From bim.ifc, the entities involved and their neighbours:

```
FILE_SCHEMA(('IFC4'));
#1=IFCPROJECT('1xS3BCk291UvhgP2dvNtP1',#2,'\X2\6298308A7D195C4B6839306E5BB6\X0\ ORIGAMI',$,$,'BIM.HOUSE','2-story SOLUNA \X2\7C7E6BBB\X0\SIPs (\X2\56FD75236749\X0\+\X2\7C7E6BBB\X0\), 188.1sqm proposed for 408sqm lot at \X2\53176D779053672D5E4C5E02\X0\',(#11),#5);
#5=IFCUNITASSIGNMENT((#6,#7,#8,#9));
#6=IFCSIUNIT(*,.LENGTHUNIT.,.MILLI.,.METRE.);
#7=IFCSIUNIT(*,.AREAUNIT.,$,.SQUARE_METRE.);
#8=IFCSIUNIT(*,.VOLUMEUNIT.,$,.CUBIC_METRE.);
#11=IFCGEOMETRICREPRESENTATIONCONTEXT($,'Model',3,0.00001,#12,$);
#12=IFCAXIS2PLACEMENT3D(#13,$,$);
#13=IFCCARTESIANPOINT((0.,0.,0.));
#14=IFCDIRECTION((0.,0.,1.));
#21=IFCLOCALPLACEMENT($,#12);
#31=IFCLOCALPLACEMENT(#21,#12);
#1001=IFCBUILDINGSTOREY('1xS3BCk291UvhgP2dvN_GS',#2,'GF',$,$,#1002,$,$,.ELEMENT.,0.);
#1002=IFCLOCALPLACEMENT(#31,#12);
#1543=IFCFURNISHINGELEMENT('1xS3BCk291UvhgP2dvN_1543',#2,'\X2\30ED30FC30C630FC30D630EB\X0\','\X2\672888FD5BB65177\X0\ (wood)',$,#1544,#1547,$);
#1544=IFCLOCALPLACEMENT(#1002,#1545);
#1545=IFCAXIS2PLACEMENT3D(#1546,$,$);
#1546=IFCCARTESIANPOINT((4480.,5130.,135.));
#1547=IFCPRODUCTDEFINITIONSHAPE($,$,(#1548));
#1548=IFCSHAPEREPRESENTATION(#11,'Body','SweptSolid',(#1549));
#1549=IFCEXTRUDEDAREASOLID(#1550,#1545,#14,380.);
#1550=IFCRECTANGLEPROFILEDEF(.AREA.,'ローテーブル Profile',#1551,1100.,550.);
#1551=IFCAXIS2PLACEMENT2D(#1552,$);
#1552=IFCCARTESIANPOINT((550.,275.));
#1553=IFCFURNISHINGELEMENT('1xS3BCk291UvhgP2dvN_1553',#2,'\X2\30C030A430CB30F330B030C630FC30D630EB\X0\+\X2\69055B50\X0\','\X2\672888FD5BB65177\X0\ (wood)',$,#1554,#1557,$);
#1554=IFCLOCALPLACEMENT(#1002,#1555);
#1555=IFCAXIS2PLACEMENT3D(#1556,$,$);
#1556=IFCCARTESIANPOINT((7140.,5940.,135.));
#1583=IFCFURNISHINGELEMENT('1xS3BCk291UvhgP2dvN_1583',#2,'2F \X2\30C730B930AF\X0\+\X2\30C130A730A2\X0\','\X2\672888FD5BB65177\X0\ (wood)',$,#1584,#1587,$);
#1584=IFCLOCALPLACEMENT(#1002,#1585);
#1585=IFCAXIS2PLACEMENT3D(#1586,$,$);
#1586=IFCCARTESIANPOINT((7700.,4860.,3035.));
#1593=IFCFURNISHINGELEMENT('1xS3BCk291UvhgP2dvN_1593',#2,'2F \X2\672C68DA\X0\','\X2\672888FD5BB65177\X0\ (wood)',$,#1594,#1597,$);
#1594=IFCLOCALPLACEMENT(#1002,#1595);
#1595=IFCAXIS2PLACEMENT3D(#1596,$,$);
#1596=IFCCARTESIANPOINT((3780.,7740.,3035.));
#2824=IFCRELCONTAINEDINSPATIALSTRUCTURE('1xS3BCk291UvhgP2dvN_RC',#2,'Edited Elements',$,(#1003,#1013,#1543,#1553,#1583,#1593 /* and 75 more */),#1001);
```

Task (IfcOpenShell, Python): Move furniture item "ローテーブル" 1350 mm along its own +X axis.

```python
import ifcopenshell
import ifcopenshell.api.geometry
import ifcopenshell.util.placement
import ifcopenshell.util.unit

model = ifcopenshell.open("bim.ifc")
unit_scale = ifcopenshell.util.unit.calculate_unit_scale(model)

item = model.by_id(1543)
matrix = ifcopenshell.util.placement.get_local_placement(item.ObjectPlacement)
matrix[:3, 3] += matrix[:3, 0] * 1.35 / unit_scale
ifcopenshell.api.geometry.edit_object_placement(model, product=item, matrix=matrix, is_si=False)

print(ifcopenshell.util.placement.get_local_placement(item.ObjectPlacement).round(3) + 0.0)

model.write("bim_rev.ifc")
```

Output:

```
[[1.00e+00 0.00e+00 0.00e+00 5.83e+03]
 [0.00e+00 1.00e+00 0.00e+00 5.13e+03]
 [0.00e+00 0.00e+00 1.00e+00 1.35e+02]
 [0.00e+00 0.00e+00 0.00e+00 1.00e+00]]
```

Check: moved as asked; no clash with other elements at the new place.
